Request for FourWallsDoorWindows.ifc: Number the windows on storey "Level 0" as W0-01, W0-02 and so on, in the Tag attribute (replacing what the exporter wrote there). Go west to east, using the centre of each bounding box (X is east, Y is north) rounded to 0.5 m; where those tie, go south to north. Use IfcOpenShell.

First a look at what the model holds.

```python
import ifcopenshell
import ifcopenshell.util.element
import ifcopenshell.util.placement

model = ifcopenshell.open("FourWallsDoorWindows.ifc")
print(model.schema)
storey = next(s for s in model.by_type("IfcBuildingStorey") if s.Name == "Level 0")
windows = [e for e in ifcopenshell.util.element.get_decomposition(storey) if e.is_a("IfcWindow")]
for e in sorted(windows, key=lambda e: e.id()):
    origin = ifcopenshell.util.placement.get_local_placement(e.ObjectPlacement)[:3, 3]
    print(e.id(), e.Tag, e.Name, origin.round(2) + 0.0, sep=" | ")
```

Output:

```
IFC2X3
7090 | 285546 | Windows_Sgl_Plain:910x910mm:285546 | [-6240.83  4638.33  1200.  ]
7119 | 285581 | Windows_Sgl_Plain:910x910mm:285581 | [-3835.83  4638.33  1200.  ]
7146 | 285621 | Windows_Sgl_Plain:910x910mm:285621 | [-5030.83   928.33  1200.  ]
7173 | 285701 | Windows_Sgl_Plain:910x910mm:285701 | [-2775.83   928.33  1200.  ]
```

```python
import ifcopenshell
import ifcopenshell.geom
import ifcopenshell.util.element
import ifcopenshell.util.shape

model = ifcopenshell.open("FourWallsDoorWindows.ifc")
settings = ifcopenshell.geom.settings()
settings.set("use-world-coords", True)


def centre(element):
    shape = ifcopenshell.geom.create_shape(settings, element)
    return ifcopenshell.util.shape.get_bbox_centroid(shape.geometry)


storey = next(s for s in model.by_type("IfcBuildingStorey") if s.Name == "Level 0")
windows = [e for e in ifcopenshell.util.element.get_decomposition(storey) if e.is_a("IfcWindow")]

# Insertion points can sit at a corner or the storey origin, so sort by the geometry (in metres).
centres = {e: centre(e) for e in windows}
windows.sort(key=lambda e: (round(centres[e][0] / 0.5), centres[e][1]))

for i, e in enumerate(windows, start=1):
    number = f"W0-{i:02d}"
    e.Tag = number
    print(e.id(), number)

model.write("FourWallsDoorWindows-out.ifc")
```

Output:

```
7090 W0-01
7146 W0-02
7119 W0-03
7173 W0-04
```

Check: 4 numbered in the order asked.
